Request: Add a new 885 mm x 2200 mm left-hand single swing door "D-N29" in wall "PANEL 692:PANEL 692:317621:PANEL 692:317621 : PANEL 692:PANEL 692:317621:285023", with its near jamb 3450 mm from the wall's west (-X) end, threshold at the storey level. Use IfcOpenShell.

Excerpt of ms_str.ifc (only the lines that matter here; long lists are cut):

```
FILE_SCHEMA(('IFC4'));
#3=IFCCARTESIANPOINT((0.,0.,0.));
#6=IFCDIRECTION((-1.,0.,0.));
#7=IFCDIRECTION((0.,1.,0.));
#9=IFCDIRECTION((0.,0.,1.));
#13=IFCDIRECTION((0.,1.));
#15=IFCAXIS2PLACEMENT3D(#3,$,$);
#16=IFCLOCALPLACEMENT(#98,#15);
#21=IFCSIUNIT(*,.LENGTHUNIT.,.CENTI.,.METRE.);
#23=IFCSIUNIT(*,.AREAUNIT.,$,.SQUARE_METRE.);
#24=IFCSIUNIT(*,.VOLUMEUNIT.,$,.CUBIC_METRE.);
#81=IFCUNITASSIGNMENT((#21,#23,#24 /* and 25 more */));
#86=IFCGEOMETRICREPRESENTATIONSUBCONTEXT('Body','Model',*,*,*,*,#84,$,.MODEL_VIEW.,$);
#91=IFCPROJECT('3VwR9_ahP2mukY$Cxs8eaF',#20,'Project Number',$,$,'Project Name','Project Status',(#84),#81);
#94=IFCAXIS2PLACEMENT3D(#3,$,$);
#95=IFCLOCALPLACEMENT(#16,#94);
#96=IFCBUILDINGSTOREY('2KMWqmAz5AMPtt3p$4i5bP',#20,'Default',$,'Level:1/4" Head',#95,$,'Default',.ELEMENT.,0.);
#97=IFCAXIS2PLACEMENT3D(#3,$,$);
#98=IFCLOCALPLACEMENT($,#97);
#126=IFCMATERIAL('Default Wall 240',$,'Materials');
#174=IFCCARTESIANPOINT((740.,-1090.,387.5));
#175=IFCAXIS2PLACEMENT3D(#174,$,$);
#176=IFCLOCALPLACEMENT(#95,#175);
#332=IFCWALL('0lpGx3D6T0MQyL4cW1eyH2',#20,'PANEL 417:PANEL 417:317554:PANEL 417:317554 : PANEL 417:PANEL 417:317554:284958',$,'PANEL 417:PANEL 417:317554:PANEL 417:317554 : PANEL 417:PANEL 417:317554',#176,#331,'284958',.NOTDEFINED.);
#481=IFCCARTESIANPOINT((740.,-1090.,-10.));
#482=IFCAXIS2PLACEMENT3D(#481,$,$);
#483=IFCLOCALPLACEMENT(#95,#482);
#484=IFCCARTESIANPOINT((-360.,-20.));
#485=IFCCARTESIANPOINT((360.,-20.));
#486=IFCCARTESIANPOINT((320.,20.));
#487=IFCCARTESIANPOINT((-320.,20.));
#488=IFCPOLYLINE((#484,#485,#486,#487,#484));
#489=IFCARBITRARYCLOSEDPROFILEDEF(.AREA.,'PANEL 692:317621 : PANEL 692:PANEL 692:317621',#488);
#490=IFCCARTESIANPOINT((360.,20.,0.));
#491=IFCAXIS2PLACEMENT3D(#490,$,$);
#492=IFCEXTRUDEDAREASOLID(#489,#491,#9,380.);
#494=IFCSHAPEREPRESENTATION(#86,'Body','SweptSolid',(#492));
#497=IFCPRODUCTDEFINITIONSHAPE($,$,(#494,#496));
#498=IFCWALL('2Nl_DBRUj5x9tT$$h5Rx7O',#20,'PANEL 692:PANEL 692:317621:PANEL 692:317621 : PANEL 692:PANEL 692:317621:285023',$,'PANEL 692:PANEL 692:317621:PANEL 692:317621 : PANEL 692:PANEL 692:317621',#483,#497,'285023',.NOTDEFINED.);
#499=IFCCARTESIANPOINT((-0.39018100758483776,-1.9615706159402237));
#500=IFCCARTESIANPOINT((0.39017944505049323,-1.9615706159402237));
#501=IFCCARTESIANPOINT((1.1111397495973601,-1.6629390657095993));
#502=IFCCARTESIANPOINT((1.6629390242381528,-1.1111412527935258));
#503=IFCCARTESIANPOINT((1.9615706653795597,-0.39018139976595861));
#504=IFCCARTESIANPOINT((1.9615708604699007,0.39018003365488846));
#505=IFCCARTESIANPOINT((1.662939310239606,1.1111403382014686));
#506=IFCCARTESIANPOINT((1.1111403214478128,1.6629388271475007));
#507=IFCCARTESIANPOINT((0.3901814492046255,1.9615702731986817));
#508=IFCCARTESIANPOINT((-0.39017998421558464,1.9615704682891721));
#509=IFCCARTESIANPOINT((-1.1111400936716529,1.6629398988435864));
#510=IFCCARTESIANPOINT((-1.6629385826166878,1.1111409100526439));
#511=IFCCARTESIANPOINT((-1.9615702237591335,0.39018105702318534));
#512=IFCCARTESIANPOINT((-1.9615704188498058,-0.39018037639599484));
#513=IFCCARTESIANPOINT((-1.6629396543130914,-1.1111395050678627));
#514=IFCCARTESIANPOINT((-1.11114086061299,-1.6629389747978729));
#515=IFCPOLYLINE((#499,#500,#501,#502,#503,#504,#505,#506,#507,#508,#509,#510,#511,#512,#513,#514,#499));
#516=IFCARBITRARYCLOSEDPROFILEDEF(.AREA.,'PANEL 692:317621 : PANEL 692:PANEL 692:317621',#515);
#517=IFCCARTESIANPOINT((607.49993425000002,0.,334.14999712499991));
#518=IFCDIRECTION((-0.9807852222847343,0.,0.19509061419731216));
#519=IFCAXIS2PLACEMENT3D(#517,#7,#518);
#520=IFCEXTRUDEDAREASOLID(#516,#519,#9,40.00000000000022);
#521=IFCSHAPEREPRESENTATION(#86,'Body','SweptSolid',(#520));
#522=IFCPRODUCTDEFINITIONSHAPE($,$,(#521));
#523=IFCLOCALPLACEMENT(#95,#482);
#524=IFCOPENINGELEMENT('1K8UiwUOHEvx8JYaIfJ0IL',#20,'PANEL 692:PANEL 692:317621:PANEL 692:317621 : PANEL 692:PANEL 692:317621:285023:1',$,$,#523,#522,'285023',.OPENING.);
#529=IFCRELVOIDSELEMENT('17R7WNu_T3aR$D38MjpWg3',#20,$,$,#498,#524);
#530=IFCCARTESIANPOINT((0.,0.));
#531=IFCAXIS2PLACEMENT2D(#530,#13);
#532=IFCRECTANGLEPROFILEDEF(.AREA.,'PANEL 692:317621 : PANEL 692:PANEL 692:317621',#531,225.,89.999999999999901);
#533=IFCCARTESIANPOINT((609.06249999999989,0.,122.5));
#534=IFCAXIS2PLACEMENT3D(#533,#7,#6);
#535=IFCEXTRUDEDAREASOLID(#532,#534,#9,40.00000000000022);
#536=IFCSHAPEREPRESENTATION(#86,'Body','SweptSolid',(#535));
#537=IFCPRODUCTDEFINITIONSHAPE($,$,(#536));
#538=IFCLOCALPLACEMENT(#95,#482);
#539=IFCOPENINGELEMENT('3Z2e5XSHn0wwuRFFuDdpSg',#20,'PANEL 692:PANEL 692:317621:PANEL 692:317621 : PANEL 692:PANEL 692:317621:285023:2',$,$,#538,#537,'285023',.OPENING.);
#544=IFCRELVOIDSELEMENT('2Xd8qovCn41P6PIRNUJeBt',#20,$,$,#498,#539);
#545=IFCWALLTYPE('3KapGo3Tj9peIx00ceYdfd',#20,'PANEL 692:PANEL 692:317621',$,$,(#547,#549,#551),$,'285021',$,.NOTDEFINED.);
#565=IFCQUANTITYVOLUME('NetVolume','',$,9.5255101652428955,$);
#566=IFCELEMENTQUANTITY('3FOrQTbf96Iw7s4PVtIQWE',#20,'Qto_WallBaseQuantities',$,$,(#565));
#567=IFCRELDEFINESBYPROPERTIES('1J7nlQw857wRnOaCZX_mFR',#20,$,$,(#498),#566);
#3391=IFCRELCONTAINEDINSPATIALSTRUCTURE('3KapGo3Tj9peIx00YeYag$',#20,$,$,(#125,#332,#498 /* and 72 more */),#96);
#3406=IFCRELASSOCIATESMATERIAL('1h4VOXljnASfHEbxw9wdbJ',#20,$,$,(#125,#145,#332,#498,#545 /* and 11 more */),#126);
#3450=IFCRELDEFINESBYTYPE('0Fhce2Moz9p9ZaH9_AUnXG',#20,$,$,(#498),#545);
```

```python
import numpy as np
import ifcopenshell
import ifcopenshell.api.feature
import ifcopenshell.api.geometry
import ifcopenshell.api.pset
import ifcopenshell.api.root
import ifcopenshell.api.spatial
import ifcopenshell.geom
import ifcopenshell.util.element
import ifcopenshell.util.placement
import ifcopenshell.util.representation
import ifcopenshell.util.shape
import ifcopenshell.util.unit

model = ifcopenshell.open("ms_str.ifc")
unit_scale = ifcopenshell.util.unit.calculate_unit_scale(model)
volume_scale = ifcopenshell.util.unit.calculate_unit_scale(model, "VOLUMEUNIT")
settings = ifcopenshell.geom.settings()


def volume(element):
    """Net volume in cubic metres, openings subtracted."""
    shape = ifcopenshell.geom.create_shape(settings, element)
    return ifcopenshell.util.shape.get_volume(shape.geometry)


wall = model.by_guid("2Nl_DBRUj5x9tT$$h5Rx7O")
storey = ifcopenshell.util.element.get_container(wall, ifc_class="IfcBuildingStorey")
context = ifcopenshell.util.representation.get_context(model, "Model", "Body", "MODEL_VIEW")
before = volume(wall)

width, height, from_end, sill = 0.885, 2.2, 3.45, 0.0  # metres

# The wall runs along its own X axis, and the end named is its -X end.
wall_shape = ifcopenshell.geom.create_shape(settings, wall)
x, y, z = ifcopenshell.util.shape.get_vertices(wall_shape.geometry).T
start = x.min() + from_end
face, thickness = float(y.min()), float(y.max() - y.min())
wall_matrix = ifcopenshell.util.placement.get_local_placement(wall.ObjectPlacement)
level = ifcopenshell.util.placement.get_local_placement(storey.ObjectPlacement)[2, 3]


def in_wall(x, y):
    """Placement at x, y metres in the wall's axes, at sill height."""
    matrix = wall_matrix.copy()
    matrix[:, 3] = wall_matrix @ np.array([x / unit_scale, y / unit_scale, 0.0, 1.0])
    matrix[2, 3] = level + sill / unit_scale
    return matrix


# Opening: a box that overshoots both wall faces by 50 mm.
opening = ifcopenshell.api.root.create_entity(model, ifc_class="IfcOpeningElement", predefined_type="OPENING")
box = ifcopenshell.api.geometry.add_wall_representation(
    model, context=context, length=width, height=height, thickness=thickness + 0.1
)
ifcopenshell.api.geometry.assign_representation(model, product=opening, representation=box)
ifcopenshell.api.geometry.edit_object_placement(model, product=opening, matrix=in_wall(start, face - 0.05), is_si=False)
ifcopenshell.api.feature.add_feature(model, feature=opening, element=wall)

door = ifcopenshell.api.root.create_entity(model, ifc_class="IfcDoor", name="D-N29", predefined_type="DOOR")
door.OverallWidth, door.OverallHeight = width / unit_scale, height / unit_scale
door.OperationType = "SINGLE_SWING_LEFT"
body = ifcopenshell.api.geometry.add_door_representation(
    model,
    context=context,
    overall_width=door.OverallWidth,
    overall_height=door.OverallHeight,
    operation_type="SINGLE_SWING_LEFT",
    lining_properties={"LiningDepth": thickness / unit_scale, "ThresholdDepth": thickness / unit_scale},
)
ifcopenshell.api.geometry.assign_representation(model, product=door, representation=body)
ifcopenshell.api.spatial.assign_container(model, products=[door], relating_structure=storey)
ifcopenshell.api.feature.add_filling(model, opening=opening, element=door)

# The lining spans the wall, so the door starts at the wall face.
ifcopenshell.api.geometry.edit_object_placement(model, product=door, matrix=in_wall(start, face), is_si=False)

after = volume(wall)

# Update the wall's stored quantities.
qto = model.by_id(ifcopenshell.util.element.get_pset(wall, "Qto_WallBaseQuantities", should_inherit=False)["id"])
ifcopenshell.api.pset.edit_qto(model, qto=qto, properties={"NetVolume": after / volume_scale})

print(f"wall volume {before:.3f} -> {after:.3f} m3")

model.write("ms_str_rev.ifc")
```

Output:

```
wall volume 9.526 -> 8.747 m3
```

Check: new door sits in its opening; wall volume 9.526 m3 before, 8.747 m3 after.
